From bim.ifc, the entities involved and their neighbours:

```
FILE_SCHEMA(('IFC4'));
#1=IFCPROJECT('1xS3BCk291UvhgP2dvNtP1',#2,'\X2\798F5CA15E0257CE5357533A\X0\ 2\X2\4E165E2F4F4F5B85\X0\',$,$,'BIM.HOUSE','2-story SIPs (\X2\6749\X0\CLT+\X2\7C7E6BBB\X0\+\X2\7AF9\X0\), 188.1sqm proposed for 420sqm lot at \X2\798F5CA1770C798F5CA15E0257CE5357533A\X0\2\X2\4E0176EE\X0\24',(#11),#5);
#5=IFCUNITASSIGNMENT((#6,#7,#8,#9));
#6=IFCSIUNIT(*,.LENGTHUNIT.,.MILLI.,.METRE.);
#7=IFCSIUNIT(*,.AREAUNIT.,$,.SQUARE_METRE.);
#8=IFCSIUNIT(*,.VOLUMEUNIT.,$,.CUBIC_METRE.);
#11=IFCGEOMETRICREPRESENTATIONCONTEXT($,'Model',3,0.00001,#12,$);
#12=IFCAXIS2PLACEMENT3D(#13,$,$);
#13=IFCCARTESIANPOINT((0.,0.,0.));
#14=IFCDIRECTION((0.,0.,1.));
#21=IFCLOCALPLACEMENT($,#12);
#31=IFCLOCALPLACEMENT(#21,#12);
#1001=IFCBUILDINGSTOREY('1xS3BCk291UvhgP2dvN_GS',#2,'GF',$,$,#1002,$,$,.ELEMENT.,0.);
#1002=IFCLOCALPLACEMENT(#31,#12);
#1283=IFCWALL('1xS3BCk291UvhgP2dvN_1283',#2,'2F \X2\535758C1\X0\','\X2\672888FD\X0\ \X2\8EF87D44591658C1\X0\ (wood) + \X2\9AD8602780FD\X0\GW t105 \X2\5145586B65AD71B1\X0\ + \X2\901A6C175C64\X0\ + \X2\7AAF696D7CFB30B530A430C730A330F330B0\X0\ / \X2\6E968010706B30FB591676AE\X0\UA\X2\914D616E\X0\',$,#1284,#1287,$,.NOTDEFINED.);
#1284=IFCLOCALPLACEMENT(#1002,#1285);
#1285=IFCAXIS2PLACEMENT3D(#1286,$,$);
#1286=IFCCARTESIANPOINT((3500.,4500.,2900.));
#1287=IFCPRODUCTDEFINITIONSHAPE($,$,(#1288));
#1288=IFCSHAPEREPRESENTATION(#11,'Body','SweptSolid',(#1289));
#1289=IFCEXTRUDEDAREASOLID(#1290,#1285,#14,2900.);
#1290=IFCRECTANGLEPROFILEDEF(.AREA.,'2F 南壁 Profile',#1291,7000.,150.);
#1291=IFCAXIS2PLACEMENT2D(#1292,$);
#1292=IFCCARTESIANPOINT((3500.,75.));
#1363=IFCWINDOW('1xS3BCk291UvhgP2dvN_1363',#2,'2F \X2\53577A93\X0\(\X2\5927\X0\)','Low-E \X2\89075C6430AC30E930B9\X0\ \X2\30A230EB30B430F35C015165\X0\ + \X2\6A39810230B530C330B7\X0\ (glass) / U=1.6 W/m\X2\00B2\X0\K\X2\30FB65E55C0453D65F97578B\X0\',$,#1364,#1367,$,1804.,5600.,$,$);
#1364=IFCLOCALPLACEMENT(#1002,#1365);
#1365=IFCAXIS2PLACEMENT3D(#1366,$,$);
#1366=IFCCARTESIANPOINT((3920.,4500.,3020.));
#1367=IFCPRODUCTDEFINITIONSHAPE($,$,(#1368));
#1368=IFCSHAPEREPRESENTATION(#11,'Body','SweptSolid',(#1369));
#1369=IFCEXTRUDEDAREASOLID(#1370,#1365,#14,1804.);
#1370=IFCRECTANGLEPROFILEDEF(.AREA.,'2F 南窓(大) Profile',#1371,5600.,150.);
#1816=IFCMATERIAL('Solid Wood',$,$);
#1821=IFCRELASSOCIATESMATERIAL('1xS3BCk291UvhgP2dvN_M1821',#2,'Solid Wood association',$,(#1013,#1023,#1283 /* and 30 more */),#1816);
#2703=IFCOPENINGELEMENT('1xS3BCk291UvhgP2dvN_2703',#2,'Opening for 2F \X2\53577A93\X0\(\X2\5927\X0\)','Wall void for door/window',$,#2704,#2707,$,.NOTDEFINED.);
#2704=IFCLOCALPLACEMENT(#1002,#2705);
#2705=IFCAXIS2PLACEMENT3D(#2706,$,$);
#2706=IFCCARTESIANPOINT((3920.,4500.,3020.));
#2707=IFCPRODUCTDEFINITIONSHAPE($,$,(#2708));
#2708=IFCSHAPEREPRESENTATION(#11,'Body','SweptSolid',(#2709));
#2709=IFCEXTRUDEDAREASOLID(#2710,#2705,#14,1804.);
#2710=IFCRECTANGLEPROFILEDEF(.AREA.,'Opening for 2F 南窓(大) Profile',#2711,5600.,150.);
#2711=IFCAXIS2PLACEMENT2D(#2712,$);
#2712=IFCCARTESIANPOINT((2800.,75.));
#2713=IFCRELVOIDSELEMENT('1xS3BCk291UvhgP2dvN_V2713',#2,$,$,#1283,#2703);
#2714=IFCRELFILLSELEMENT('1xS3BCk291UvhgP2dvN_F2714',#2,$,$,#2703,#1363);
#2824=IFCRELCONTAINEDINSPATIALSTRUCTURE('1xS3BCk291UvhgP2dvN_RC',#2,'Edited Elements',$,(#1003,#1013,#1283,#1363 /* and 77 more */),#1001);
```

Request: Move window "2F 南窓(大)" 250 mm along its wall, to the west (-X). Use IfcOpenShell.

```python
import ifcopenshell
import ifcopenshell.api.geometry
import ifcopenshell.util.placement

model = ifcopenshell.open("bim.ifc")

window = model.by_id(1363)
opening = window.FillsVoids[0].RelatingOpeningElement
wall = opening.VoidsElements[0].RelatingBuildingElement

wall_matrix = ifcopenshell.util.placement.get_local_placement(wall.ObjectPlacement)
shift = wall_matrix[:3, 0] * -250.0
before = ifcopenshell.util.placement.get_local_placement(window.ObjectPlacement)[:3, 3].copy()

# The window is not placed relative to its opening, so move both.
for product in (opening, window):
    matrix = ifcopenshell.util.placement.get_local_placement(product.ObjectPlacement)
    matrix[:3, 3] += shift
    ifcopenshell.api.geometry.edit_object_placement(model, product=product, matrix=matrix, is_si=False)

after = ifcopenshell.util.placement.get_local_placement(window.ObjectPlacement)[:3, 3]
print("window moved by", (after - before).round(3) + 0.0)

model.write("bim-out.ifc")
```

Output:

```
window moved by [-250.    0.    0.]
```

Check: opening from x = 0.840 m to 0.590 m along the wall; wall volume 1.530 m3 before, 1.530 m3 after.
